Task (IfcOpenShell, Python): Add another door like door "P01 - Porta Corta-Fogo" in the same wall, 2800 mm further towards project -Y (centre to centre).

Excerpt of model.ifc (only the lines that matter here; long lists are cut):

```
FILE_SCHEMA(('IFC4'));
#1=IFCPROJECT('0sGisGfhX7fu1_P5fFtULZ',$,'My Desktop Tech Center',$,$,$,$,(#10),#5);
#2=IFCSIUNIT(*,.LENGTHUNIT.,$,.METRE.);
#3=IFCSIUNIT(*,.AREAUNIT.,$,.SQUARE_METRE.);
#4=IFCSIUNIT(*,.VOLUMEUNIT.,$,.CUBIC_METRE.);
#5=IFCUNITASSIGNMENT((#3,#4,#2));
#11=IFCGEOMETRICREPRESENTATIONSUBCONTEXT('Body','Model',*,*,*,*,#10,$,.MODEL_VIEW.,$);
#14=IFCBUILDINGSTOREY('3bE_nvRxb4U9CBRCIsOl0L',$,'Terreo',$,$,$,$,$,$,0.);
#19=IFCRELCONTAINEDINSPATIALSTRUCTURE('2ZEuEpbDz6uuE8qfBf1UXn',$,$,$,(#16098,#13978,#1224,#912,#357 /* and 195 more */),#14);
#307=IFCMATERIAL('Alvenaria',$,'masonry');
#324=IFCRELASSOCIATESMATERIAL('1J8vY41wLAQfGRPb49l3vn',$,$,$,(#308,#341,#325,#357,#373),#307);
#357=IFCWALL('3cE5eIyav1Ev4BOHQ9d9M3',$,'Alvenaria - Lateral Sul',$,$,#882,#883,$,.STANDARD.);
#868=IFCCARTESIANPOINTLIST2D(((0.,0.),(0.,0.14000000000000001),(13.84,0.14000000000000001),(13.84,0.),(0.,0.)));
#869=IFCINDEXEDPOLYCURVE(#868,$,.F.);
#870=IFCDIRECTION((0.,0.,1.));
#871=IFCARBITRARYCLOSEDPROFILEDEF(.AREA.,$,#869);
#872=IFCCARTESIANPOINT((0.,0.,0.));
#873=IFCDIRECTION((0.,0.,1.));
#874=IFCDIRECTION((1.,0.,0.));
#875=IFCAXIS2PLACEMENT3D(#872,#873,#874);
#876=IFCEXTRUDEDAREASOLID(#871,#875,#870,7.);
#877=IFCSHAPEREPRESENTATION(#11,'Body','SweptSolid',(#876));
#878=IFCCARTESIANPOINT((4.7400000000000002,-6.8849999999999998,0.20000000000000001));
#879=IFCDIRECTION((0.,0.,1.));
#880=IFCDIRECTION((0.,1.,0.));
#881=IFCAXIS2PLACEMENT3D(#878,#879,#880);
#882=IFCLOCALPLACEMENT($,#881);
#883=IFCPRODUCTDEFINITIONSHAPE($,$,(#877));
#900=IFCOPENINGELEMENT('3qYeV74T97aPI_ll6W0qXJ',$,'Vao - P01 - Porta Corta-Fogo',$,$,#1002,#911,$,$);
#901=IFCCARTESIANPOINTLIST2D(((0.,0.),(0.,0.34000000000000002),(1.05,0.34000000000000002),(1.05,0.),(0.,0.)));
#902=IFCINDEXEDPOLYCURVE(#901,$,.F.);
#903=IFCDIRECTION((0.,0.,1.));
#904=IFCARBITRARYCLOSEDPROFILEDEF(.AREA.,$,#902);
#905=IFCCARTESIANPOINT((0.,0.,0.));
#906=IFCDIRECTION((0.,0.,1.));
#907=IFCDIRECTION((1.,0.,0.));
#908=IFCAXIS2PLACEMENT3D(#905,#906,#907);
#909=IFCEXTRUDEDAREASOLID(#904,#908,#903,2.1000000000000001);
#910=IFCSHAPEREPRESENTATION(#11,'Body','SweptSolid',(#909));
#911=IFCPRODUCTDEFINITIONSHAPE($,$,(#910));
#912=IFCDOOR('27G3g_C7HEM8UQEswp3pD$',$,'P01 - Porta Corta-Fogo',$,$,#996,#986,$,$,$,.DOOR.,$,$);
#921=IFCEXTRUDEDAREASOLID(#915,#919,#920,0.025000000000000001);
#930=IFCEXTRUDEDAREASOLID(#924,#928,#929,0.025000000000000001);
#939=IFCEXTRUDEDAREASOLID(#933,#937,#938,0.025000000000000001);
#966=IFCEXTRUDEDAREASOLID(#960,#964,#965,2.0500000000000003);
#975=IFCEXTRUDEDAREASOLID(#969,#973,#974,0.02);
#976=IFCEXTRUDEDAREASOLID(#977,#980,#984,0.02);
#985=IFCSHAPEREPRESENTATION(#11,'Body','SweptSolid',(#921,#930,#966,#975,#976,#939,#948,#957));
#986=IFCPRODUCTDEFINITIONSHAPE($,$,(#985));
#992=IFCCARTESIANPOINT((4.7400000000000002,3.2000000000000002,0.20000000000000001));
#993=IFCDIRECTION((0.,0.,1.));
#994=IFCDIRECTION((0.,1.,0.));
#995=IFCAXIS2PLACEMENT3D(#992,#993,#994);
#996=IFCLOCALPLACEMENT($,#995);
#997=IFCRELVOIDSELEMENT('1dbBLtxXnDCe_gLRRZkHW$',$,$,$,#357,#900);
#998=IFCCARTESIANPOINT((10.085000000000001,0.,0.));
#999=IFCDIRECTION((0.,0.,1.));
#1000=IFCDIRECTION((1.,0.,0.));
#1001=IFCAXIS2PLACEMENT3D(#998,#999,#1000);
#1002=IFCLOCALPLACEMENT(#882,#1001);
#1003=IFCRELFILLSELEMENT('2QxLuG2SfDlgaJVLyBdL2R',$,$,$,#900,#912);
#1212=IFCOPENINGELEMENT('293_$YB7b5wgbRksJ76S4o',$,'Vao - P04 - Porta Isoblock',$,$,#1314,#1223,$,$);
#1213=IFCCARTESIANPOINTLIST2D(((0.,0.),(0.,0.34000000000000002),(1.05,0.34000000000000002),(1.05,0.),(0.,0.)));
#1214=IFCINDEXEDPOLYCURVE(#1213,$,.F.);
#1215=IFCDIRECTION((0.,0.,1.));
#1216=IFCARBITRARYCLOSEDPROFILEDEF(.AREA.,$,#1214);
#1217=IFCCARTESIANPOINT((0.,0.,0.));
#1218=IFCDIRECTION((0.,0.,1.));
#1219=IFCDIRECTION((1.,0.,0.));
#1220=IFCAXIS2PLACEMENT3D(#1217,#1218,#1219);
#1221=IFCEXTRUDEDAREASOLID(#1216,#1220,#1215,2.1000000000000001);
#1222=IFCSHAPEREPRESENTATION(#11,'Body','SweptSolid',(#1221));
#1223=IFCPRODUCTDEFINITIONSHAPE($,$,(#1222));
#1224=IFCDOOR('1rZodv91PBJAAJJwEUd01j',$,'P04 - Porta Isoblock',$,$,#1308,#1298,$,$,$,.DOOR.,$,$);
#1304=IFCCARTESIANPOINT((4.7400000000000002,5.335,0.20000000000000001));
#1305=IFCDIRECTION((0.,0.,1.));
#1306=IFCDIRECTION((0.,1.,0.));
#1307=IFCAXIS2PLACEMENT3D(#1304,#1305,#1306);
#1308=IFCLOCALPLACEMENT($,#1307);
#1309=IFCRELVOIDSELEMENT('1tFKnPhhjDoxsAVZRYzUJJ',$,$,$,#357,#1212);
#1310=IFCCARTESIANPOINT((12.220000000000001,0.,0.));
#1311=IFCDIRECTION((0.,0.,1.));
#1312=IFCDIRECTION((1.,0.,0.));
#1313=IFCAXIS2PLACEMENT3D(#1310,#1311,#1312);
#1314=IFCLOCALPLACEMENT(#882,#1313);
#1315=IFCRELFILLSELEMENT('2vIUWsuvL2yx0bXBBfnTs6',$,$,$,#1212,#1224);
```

```python
import ifcopenshell
import ifcopenshell.api.feature
import ifcopenshell.api.geometry
import ifcopenshell.api.root
import ifcopenshell.geom
import ifcopenshell.util.element
import ifcopenshell.util.placement
import ifcopenshell.util.shape
import ifcopenshell.util.unit

model = ifcopenshell.open("model.ifc")
unit_scale = ifcopenshell.util.unit.calculate_unit_scale(model)
settings = ifcopenshell.geom.settings()


def volume(element):
    """Net volume in cubic metres, openings subtracted."""
    shape = ifcopenshell.geom.create_shape(settings, element)
    return ifcopenshell.util.shape.get_volume(shape.geometry)


door = model.by_guid("27G3g_C7HEM8UQEswp3pD$")
opening = door.FillsVoids[0].RelatingOpeningElement
wall = opening.VoidsElements[0].RelatingBuildingElement
before = volume(wall)
shift = ifcopenshell.util.placement.get_local_placement(wall.ObjectPlacement)[:3, 0] * -2.8 / unit_scale

# copy_class copies the void relationship, type, container and properties, but no geometry.
new_opening = ifcopenshell.api.root.copy_class(model, product=opening)
new_opening.Representation = ifcopenshell.util.element.copy_deep(
    model, opening.Representation, exclude=["IfcGeometricRepresentationContext", "IfcRepresentationMap"]
)
new_door = ifcopenshell.api.root.copy_class(model, product=door)
new_door.Representation = ifcopenshell.util.element.copy_deep(
    model, door.Representation, exclude=["IfcGeometricRepresentationContext", "IfcRepresentationMap"]
)
ifcopenshell.api.feature.add_filling(model, opening=new_opening, element=new_door)

for old, new in ((opening, new_opening), (door, new_door)):
    matrix = ifcopenshell.util.placement.get_local_placement(old.ObjectPlacement)
    matrix[:3, 3] += shift
    ifcopenshell.api.geometry.edit_object_placement(model, product=new, matrix=matrix, is_si=False)

after = volume(wall)

print(f"wall volume {before:.3f} -> {after:.3f} m3")

model.write("model_rev.ifc")
```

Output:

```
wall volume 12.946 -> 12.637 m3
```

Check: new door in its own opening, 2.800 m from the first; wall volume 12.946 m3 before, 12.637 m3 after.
